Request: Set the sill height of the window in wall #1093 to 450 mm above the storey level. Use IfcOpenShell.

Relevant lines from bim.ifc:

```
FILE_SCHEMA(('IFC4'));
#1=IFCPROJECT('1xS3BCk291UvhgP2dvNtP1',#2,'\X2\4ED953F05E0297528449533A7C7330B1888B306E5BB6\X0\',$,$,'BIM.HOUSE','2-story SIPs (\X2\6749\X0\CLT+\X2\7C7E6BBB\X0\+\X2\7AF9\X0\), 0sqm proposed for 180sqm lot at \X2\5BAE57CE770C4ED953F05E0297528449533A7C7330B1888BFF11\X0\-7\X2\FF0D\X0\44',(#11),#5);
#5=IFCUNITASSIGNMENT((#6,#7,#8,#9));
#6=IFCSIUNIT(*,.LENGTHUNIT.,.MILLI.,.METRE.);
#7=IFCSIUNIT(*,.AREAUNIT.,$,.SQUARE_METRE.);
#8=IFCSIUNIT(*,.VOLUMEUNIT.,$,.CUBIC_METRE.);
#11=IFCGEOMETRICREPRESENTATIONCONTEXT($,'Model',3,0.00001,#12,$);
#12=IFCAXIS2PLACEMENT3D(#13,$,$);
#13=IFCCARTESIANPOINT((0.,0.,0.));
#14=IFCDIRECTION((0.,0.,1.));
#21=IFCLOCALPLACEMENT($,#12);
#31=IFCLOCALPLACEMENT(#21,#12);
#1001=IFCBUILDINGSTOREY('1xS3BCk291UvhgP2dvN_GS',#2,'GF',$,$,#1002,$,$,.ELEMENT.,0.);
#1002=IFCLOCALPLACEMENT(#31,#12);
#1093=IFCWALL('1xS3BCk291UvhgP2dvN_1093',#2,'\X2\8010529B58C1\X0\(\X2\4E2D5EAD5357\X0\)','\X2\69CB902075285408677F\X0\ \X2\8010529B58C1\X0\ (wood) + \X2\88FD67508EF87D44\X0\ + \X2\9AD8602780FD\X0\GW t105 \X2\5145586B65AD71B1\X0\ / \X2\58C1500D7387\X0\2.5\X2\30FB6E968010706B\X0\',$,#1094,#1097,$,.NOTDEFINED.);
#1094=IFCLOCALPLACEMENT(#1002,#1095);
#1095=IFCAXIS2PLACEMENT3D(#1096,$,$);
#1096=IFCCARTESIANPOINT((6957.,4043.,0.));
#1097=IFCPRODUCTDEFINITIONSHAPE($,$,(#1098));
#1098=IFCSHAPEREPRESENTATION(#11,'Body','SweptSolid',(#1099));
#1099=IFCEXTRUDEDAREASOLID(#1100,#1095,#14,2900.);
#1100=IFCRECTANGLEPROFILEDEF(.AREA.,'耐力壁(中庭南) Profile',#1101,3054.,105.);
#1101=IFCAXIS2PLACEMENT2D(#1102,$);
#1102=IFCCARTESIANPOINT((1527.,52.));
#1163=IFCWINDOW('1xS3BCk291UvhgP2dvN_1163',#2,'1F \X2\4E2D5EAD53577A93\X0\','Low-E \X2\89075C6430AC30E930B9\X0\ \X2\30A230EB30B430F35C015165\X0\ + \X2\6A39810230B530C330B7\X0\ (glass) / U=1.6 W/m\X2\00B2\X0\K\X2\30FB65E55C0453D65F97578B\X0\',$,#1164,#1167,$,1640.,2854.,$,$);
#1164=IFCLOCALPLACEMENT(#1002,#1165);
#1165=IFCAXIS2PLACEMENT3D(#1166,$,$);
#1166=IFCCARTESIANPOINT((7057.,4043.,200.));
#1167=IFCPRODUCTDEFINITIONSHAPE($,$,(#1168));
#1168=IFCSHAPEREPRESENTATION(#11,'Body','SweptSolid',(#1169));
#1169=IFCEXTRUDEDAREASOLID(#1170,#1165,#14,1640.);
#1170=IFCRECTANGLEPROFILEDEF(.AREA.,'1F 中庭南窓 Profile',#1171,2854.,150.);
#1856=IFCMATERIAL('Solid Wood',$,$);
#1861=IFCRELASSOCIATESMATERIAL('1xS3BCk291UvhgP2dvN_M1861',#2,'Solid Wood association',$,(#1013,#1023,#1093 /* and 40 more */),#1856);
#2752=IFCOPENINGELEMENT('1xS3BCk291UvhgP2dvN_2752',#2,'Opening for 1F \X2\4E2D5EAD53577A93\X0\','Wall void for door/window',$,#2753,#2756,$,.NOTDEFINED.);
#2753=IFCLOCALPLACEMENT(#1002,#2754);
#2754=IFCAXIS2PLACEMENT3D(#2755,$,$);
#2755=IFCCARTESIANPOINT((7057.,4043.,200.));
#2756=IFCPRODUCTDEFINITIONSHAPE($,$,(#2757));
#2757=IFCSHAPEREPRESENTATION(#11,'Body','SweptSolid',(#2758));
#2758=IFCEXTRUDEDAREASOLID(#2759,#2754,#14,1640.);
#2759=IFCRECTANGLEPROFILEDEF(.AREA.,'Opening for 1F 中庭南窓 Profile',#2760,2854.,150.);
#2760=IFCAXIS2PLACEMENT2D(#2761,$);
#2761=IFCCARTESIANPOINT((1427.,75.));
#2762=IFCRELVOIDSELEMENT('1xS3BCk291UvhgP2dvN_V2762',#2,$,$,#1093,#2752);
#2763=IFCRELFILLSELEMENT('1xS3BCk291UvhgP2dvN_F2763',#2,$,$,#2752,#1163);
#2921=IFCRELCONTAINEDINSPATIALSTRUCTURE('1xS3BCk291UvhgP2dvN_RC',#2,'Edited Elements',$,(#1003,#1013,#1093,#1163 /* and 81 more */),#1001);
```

```python
import numpy as np
import ifcopenshell
import ifcopenshell.api.geometry
import ifcopenshell.geom
import ifcopenshell.util.element
import ifcopenshell.util.placement
import ifcopenshell.util.shape
import ifcopenshell.util.unit

model = ifcopenshell.open("bim.ifc")
unit_scale = ifcopenshell.util.unit.calculate_unit_scale(model)

window = model.by_guid("1xS3BCk291UvhgP2dvN_1163")
opening = window.FillsVoids[0].RelatingOpeningElement
storey = ifcopenshell.util.element.get_container(window, ifc_class="IfcBuildingStorey")
level = ifcopenshell.util.placement.get_local_placement(storey.ObjectPlacement)[2, 3]

# The opening's origin need not be at the sill, so measure its lowest point.
shape = ifcopenshell.geom.create_shape(ifcopenshell.geom.settings(), opening)
bottom = ifcopenshell.util.shape.get_shape_bottom_elevation(shape, shape.geometry) / unit_scale
dz = level + 450.0 - bottom

shift = np.array([0.0, 0.0, dz])
# The window is not placed relative to its opening, so move both.
for product in (opening, window):
    matrix = ifcopenshell.util.placement.get_local_placement(product.ObjectPlacement)
    matrix[:3, 3] += shift
    ifcopenshell.api.geometry.edit_object_placement(model, product=product, matrix=matrix, is_si=False)

print(f"moved by {dz * unit_scale:+.3f} m")

model.write("bim_updated.ifc")
```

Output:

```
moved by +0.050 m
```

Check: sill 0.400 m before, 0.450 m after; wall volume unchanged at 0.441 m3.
